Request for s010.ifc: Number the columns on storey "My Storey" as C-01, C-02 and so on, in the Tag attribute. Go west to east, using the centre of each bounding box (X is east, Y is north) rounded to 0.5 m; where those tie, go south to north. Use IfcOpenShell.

First a look at what the model holds.

```python
import ifcopenshell
import ifcopenshell.util.element
import ifcopenshell.util.placement

model = ifcopenshell.open("s010.ifc")
print(model.schema)
storey = next(s for s in model.by_type("IfcBuildingStorey") if s.Name == "My Storey")
columns = [e for e in ifcopenshell.util.element.get_decomposition(storey) if e.is_a("IfcColumn")]
for e in sorted(columns, key=lambda e: e.id()):
    origin = ifcopenshell.util.placement.get_local_placement(e.ObjectPlacement)[:3, 3]
    print(e.id(), e.Tag, e.Name, origin.round(2) + 0.0, sep=" | ")
```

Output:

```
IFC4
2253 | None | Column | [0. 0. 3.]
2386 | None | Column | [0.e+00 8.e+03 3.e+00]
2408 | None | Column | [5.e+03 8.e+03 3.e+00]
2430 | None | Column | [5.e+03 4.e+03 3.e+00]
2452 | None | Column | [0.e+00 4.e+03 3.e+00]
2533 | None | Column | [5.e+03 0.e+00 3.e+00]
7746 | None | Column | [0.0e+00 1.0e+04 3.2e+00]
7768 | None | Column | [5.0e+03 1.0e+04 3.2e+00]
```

```python
import ifcopenshell
import ifcopenshell.geom
import ifcopenshell.util.element
import ifcopenshell.util.shape

model = ifcopenshell.open("s010.ifc")
settings = ifcopenshell.geom.settings()
settings.set("use-world-coords", True)


def centre(element):
    shape = ifcopenshell.geom.create_shape(settings, element)
    return ifcopenshell.util.shape.get_bbox_centroid(shape.geometry)


storey = next(s for s in model.by_type("IfcBuildingStorey") if s.Name == "My Storey")
columns = [e for e in ifcopenshell.util.element.get_decomposition(storey) if e.is_a("IfcColumn")]

# Insertion points can sit at a corner or the storey origin, so sort by the geometry (in metres).
centres = {e: centre(e) for e in columns}
columns.sort(key=lambda e: (round(centres[e][0] / 0.5), centres[e][1]))

for i, e in enumerate(columns, start=1):
    number = f"C-{i:02d}"
    e.Tag = number
    print(e.id(), number)

model.write("s010_updated.ifc")
```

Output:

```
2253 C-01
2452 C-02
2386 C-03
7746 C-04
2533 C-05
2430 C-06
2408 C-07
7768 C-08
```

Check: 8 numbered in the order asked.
